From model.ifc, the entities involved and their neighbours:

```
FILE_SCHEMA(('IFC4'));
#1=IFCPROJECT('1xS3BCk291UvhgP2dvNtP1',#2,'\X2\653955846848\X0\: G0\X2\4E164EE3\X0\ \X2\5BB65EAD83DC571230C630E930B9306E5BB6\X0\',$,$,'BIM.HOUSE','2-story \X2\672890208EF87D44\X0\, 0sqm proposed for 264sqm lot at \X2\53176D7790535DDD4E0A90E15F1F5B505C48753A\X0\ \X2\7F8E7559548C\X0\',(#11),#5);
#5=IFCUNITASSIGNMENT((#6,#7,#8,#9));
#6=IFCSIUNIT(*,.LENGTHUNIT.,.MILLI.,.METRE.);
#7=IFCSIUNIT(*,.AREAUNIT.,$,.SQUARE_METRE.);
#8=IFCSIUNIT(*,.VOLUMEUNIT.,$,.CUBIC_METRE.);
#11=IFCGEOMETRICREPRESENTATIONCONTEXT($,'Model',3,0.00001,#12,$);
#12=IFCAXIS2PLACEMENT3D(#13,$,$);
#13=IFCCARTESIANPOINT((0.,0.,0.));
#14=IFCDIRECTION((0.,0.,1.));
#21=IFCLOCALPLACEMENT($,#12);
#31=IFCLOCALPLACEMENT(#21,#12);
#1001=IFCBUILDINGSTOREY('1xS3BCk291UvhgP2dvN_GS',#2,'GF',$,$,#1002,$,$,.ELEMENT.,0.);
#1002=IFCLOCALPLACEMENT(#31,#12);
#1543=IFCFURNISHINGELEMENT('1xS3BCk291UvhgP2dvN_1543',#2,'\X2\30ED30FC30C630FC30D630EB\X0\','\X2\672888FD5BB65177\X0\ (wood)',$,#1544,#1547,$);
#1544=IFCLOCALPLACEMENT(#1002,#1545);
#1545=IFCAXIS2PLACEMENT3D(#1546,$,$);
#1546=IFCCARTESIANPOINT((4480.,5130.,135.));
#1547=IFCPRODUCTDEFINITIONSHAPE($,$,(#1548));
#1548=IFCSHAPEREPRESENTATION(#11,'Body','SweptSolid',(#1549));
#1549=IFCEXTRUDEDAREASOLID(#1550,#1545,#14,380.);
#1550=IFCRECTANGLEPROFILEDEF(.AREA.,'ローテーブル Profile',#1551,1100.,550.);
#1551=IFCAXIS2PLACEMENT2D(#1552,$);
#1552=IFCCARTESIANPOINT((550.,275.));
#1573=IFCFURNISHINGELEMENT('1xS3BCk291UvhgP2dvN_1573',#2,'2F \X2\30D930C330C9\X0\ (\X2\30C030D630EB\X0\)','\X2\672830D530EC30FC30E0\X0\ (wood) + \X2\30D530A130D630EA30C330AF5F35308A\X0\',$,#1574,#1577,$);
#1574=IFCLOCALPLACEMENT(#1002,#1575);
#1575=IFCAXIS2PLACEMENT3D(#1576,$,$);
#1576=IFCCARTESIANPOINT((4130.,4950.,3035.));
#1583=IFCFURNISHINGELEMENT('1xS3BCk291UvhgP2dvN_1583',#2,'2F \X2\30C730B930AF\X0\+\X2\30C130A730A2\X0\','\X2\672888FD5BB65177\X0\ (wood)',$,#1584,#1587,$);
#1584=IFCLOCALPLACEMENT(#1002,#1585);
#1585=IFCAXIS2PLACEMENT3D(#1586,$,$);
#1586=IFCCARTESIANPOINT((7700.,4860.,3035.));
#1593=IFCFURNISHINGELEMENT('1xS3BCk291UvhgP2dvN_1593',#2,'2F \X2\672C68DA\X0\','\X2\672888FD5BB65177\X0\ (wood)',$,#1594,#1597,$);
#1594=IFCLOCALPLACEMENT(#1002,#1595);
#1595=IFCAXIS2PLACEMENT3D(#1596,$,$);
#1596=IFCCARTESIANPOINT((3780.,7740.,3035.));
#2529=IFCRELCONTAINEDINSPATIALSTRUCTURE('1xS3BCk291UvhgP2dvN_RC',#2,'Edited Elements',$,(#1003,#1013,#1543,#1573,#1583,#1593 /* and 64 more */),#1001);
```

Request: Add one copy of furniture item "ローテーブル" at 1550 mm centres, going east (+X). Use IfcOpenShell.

```python
import numpy as np
import ifcopenshell
import ifcopenshell.api.geometry
import ifcopenshell.api.root
import ifcopenshell.util.element
import ifcopenshell.util.placement

model = ifcopenshell.open("model.ifc")


def reuse_history(source, copy):
    """copy_class also copies each property set's owner history, people and application; keep the originals."""
    for rel in copy.IsDefinedBy:
        if rel.is_a("IfcRelDefinesByProperties") and (history := rel.RelatingPropertyDefinition.OwnerHistory):
            rel.RelatingPropertyDefinition.OwnerHistory = source.OwnerHistory
            ifcopenshell.util.element.remove_deep2(model, history)


source = model.by_guid("1xS3BCk291UvhgP2dvN_1543")
base = ifcopenshell.util.placement.get_local_placement(source.ObjectPlacement)
step = np.array([1.0, 0.0, 0.0]) * 1550.0

for i in range(1, 2):
    copy = ifcopenshell.api.root.copy_class(model, product=source)
    copy.Representation = ifcopenshell.util.element.copy_deep(
        model, source.Representation, exclude=["IfcGeometricRepresentationContext", "IfcRepresentationMap"]
    )
    reuse_history(source, copy)
    matrix = base.copy()
    matrix[:3, 3] += i * step
    print("added at", matrix[:3, 3].round(3) + 0.0)
    ifcopenshell.api.geometry.edit_object_placement(model, product=copy, matrix=matrix, is_si=False)

model.write("model_rev.ifc")
```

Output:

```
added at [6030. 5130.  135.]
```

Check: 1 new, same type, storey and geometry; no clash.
